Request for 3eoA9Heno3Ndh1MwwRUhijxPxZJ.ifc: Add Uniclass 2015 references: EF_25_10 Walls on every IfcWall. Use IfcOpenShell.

First a look at what the model holds.

```python
import ifcopenshell

model = ifcopenshell.open("3eoA9Heno3Ndh1MwwRUhijxPxZJ.ifc")
print(model.schema)
print("classifications:", [c.Name for c in model.by_type("IfcClassification")])
for ifc_class in ("IfcDoor", "IfcRoof", "IfcStair", "IfcWall", "IfcWindow"):
    print(ifc_class, len(model.by_type(ifc_class)))
```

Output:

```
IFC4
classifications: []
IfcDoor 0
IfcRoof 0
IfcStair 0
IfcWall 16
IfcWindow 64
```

```python
import ifcopenshell
import ifcopenshell.api.classification

model = ifcopenshell.open("3eoA9Heno3Ndh1MwwRUhijxPxZJ.ifc")

system = ifcopenshell.api.classification.add_classification(model, classification="Uniclass 2015")

codes = {
    "IfcWall": ("EF_25_10", "Walls"),
}
for ifc_class, (code, name) in codes.items():
    products = model.by_type(ifc_class)
    ifcopenshell.api.classification.add_reference(
        model, products=products, classification=system, identification=code, name=name
    )
    print(code, len(products))

model.write("3eoA9Heno3Ndh1MwwRUhijxPxZJ_v2.ifc")
```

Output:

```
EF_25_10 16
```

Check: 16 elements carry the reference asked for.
